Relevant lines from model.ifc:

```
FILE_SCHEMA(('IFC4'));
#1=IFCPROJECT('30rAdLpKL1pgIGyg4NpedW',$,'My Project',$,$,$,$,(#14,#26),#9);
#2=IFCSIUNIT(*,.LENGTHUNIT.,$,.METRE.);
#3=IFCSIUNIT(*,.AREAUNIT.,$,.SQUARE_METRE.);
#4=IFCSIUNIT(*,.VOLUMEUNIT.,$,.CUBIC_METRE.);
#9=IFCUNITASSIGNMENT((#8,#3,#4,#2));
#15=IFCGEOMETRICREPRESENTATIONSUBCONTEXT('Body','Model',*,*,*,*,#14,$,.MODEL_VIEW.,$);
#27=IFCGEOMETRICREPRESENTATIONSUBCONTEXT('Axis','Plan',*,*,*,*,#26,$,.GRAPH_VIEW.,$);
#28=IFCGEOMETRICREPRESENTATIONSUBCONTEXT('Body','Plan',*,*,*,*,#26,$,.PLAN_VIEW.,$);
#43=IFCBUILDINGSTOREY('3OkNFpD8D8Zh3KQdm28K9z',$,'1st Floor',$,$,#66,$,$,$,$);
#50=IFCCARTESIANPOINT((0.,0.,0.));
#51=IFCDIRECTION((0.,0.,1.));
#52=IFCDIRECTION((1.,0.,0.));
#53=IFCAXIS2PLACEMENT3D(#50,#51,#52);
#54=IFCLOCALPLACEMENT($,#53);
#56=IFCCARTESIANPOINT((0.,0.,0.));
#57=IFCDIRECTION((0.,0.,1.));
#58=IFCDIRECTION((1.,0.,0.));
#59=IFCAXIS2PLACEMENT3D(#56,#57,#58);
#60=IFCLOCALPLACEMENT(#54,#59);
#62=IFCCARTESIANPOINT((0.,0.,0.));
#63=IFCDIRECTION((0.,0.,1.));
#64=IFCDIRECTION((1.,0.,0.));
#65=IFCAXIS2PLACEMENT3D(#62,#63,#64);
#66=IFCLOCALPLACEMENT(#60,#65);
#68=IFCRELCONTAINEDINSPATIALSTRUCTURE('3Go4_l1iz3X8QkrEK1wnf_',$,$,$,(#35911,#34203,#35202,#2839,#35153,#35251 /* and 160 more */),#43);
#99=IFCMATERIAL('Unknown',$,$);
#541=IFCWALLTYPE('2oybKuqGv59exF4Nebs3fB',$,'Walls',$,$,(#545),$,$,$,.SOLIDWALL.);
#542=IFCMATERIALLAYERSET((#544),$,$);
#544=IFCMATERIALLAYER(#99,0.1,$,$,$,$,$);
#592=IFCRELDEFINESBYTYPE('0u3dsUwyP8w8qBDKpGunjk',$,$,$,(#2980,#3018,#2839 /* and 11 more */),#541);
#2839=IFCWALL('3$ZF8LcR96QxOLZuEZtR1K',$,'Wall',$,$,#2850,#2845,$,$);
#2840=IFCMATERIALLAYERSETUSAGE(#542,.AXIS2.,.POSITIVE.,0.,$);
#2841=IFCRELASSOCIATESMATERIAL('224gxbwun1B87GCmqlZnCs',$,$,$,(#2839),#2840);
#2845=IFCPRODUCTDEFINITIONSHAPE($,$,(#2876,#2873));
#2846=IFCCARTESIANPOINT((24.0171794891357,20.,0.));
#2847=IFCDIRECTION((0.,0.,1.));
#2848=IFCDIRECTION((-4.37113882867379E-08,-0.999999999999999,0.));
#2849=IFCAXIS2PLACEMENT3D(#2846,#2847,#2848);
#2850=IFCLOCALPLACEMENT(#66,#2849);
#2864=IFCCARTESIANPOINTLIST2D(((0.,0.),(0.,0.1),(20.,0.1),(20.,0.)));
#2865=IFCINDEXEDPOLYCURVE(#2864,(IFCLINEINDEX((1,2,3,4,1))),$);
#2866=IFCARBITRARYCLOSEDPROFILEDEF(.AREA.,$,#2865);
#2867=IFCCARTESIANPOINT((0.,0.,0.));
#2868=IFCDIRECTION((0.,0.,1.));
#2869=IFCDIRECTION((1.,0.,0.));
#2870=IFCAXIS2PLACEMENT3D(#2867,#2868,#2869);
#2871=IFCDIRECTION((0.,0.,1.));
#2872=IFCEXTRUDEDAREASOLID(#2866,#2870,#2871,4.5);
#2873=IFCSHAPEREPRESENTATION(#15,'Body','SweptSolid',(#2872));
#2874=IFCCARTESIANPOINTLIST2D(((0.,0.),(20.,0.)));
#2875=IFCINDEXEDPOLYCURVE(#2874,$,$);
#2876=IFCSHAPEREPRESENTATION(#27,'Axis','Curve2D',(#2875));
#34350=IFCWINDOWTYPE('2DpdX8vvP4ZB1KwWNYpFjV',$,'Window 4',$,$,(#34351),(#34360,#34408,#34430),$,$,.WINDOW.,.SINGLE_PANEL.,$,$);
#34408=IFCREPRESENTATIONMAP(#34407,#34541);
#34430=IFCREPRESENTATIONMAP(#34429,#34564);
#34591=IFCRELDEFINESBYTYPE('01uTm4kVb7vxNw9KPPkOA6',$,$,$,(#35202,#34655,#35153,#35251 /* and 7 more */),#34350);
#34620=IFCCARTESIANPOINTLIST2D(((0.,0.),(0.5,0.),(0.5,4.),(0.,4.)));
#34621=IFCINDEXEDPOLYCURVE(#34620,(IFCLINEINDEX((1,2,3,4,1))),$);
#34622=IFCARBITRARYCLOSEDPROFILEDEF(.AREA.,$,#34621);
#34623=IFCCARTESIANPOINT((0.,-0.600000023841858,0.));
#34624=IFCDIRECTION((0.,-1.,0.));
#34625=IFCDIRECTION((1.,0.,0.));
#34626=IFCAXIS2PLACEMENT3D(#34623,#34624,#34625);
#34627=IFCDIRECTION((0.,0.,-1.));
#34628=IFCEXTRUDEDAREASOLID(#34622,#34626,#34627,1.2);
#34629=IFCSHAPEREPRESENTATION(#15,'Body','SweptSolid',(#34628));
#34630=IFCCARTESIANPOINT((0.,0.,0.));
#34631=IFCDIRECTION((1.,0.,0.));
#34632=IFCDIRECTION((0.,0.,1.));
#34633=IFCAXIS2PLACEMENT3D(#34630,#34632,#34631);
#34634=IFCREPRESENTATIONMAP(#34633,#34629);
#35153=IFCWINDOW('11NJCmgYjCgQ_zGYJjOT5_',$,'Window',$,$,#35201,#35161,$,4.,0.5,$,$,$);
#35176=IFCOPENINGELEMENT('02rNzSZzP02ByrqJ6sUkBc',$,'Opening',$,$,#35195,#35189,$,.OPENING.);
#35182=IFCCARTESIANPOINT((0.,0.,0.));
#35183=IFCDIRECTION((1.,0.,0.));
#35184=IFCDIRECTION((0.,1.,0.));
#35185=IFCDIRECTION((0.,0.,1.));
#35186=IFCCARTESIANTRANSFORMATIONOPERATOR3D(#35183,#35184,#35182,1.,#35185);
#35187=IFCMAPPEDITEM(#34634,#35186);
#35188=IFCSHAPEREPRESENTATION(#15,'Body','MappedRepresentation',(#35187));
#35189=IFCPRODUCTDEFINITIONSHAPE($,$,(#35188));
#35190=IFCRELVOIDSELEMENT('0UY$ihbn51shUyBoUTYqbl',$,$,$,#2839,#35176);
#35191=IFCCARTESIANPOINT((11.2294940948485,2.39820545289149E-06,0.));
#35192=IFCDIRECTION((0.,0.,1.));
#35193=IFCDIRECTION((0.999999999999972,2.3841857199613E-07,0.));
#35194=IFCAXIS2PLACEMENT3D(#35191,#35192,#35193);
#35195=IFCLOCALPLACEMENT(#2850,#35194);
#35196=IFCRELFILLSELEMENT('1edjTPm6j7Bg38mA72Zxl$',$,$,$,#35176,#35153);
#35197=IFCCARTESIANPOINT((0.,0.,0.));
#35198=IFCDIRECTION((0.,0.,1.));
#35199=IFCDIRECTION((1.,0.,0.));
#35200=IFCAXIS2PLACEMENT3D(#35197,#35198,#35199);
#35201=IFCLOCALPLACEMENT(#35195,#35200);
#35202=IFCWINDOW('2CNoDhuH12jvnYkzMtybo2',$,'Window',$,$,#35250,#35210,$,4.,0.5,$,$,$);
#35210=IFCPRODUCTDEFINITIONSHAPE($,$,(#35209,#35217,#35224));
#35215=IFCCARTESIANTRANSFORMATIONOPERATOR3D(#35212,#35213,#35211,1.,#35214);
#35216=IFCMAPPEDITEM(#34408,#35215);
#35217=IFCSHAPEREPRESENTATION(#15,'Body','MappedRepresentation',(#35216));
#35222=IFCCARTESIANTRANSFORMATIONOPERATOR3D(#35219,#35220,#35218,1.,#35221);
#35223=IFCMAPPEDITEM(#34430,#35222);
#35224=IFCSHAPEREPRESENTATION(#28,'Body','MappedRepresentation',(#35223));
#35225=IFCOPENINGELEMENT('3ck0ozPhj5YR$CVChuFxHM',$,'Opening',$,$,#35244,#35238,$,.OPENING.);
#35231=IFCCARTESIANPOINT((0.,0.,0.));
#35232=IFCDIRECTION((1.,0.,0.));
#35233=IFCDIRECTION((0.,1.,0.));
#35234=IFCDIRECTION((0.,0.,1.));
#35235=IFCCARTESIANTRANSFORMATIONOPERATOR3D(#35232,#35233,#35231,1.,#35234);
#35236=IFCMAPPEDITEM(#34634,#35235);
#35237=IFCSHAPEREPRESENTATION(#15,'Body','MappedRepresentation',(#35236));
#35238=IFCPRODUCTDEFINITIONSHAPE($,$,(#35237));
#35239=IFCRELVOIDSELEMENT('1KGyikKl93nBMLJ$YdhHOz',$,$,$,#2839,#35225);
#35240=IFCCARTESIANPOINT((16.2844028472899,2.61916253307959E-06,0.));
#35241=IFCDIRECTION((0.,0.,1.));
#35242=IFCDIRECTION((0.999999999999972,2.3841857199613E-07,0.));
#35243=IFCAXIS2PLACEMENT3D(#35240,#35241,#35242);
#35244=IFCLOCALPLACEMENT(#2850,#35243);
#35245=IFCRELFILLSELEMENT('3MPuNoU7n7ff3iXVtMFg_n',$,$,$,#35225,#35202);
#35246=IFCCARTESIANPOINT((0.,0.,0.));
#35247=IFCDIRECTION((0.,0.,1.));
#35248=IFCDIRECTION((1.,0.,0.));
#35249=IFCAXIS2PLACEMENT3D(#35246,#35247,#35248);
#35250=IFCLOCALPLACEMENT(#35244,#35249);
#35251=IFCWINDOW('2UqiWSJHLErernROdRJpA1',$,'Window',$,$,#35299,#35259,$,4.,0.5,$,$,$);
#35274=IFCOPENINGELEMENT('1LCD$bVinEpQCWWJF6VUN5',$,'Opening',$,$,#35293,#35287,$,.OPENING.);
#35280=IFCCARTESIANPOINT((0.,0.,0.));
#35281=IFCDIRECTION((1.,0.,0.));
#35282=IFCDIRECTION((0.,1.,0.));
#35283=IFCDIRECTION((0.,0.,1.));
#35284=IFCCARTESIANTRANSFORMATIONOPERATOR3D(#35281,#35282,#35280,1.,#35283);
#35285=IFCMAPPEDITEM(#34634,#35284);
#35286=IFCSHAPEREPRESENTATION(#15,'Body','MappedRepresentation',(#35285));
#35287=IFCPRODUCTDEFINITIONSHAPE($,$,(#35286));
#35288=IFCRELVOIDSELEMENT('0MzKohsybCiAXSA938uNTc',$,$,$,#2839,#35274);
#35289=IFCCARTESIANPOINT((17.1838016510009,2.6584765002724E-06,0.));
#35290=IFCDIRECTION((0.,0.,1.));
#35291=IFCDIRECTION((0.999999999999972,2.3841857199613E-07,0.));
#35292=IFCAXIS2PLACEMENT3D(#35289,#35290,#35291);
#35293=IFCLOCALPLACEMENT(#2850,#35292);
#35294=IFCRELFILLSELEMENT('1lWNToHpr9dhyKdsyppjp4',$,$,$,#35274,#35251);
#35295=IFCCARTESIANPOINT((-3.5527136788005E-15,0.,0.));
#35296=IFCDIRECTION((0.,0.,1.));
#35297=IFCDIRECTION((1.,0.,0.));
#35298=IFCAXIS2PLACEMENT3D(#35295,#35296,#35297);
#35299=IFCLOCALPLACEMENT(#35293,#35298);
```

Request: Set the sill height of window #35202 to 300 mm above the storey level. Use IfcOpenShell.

```python
import numpy as np
import ifcopenshell
import ifcopenshell.api.geometry
import ifcopenshell.geom
import ifcopenshell.util.element
import ifcopenshell.util.placement
import ifcopenshell.util.shape
import ifcopenshell.util.unit

model = ifcopenshell.open("model.ifc")
unit_scale = ifcopenshell.util.unit.calculate_unit_scale(model)

window = model.by_id(35202)
opening = window.FillsVoids[0].RelatingOpeningElement
storey = ifcopenshell.util.element.get_container(window, ifc_class="IfcBuildingStorey")
level = ifcopenshell.util.placement.get_local_placement(storey.ObjectPlacement)[2, 3]

# The opening's origin need not be at the sill, so measure its lowest point.
shape = ifcopenshell.geom.create_shape(ifcopenshell.geom.settings(), opening)
bottom = ifcopenshell.util.shape.get_shape_bottom_elevation(shape, shape.geometry) / unit_scale
dz = level + 0.3 / unit_scale - bottom

shift = np.array([0.0, 0.0, dz])
# The window is placed relative to its opening, so it follows when the opening moves.
matrix = ifcopenshell.util.placement.get_local_placement(opening.ObjectPlacement)
matrix[:3, 3] += shift
ifcopenshell.api.geometry.edit_object_placement(
    model, product=opening, matrix=matrix, is_si=False, should_transform_children=True
)

print(f"moved by {dz * unit_scale:+.3f} m")

model.write("model_updated.ifc")
```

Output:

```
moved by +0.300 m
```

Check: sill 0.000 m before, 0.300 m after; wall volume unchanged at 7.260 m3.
